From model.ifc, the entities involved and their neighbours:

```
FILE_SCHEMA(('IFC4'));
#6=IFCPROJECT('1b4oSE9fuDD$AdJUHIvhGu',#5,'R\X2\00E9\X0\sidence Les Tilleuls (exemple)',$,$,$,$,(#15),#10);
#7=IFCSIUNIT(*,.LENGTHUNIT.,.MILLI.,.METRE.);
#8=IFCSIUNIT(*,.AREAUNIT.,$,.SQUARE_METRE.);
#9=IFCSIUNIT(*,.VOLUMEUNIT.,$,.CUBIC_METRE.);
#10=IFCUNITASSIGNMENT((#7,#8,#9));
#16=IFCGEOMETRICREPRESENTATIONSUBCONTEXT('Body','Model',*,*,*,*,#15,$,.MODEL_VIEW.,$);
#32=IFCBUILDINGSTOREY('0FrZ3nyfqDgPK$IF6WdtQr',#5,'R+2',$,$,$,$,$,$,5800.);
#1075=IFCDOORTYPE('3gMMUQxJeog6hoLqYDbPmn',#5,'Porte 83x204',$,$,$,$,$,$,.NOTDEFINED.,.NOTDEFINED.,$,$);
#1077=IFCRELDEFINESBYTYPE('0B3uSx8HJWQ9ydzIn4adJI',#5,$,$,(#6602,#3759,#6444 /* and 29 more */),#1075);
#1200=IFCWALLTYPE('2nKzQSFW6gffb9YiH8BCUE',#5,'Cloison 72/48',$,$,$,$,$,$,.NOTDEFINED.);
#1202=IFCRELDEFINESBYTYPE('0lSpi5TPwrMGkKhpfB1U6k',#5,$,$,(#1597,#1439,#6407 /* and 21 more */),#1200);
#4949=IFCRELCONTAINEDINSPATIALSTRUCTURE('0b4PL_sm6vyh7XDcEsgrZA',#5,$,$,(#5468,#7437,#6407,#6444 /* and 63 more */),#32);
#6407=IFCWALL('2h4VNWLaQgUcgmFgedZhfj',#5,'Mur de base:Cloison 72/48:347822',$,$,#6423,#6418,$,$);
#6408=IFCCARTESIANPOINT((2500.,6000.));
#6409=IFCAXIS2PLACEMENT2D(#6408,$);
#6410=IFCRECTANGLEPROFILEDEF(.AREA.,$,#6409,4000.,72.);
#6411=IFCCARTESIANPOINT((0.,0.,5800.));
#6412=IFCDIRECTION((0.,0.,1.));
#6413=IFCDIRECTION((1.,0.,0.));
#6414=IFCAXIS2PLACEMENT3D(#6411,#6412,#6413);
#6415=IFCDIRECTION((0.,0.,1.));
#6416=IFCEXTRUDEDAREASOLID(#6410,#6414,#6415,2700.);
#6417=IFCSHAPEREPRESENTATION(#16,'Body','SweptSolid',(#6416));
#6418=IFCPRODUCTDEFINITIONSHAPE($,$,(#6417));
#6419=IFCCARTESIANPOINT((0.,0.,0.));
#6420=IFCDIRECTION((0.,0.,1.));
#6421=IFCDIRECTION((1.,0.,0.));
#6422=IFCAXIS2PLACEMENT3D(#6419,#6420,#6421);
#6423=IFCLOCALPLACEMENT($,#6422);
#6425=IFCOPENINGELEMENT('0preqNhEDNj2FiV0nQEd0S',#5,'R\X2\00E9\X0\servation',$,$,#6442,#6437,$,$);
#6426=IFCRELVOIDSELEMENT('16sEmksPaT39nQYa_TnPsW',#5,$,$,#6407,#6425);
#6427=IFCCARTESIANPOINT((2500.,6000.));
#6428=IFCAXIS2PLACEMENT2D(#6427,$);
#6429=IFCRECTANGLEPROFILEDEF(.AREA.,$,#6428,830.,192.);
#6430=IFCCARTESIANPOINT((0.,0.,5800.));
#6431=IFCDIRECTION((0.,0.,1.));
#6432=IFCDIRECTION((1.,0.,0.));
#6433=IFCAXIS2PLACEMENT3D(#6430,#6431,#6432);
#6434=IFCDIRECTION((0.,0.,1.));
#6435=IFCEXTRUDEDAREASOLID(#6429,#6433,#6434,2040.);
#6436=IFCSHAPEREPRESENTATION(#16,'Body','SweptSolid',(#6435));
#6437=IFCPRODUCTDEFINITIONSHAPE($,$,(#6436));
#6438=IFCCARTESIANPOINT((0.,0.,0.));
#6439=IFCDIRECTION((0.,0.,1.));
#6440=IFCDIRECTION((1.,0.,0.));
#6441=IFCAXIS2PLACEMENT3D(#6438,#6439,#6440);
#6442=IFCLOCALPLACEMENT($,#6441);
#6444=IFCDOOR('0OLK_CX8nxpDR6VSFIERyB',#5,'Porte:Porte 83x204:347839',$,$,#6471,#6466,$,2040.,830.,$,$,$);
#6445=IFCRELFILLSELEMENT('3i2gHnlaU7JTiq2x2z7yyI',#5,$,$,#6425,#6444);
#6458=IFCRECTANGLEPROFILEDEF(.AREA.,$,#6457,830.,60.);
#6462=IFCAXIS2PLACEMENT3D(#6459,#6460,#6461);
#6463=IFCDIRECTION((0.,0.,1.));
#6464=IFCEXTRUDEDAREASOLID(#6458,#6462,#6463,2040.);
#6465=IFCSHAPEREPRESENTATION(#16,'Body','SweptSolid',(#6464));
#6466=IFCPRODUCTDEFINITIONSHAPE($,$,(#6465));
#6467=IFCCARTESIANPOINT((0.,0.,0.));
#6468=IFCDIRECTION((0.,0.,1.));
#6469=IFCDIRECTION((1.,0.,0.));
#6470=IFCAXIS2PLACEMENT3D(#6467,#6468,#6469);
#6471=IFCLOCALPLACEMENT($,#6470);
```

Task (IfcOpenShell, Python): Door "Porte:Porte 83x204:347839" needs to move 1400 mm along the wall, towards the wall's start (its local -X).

```python
import ifcopenshell
import ifcopenshell.api.geometry
import ifcopenshell.util.placement

model = ifcopenshell.open("model.ifc")

door = model.by_id(6444)
opening = door.FillsVoids[0].RelatingOpeningElement
wall = opening.VoidsElements[0].RelatingBuildingElement

wall_matrix = ifcopenshell.util.placement.get_local_placement(wall.ObjectPlacement)
shift = wall_matrix[:3, 0] * -1400.0
before = ifcopenshell.util.placement.get_local_placement(door.ObjectPlacement)[:3, 3].copy()

# The door is not placed relative to its opening, so move both.
for product in (opening, door):
    matrix = ifcopenshell.util.placement.get_local_placement(product.ObjectPlacement)
    matrix[:3, 3] += shift
    ifcopenshell.api.geometry.edit_object_placement(model, product=product, matrix=matrix, is_si=False)

after = ifcopenshell.util.placement.get_local_placement(door.ObjectPlacement)[:3, 3]
print("door moved by", (after - before).round(3) + 0.0)

model.write("model_edited.ifc")
```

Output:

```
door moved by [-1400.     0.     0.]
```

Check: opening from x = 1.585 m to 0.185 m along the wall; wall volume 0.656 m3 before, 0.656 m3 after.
